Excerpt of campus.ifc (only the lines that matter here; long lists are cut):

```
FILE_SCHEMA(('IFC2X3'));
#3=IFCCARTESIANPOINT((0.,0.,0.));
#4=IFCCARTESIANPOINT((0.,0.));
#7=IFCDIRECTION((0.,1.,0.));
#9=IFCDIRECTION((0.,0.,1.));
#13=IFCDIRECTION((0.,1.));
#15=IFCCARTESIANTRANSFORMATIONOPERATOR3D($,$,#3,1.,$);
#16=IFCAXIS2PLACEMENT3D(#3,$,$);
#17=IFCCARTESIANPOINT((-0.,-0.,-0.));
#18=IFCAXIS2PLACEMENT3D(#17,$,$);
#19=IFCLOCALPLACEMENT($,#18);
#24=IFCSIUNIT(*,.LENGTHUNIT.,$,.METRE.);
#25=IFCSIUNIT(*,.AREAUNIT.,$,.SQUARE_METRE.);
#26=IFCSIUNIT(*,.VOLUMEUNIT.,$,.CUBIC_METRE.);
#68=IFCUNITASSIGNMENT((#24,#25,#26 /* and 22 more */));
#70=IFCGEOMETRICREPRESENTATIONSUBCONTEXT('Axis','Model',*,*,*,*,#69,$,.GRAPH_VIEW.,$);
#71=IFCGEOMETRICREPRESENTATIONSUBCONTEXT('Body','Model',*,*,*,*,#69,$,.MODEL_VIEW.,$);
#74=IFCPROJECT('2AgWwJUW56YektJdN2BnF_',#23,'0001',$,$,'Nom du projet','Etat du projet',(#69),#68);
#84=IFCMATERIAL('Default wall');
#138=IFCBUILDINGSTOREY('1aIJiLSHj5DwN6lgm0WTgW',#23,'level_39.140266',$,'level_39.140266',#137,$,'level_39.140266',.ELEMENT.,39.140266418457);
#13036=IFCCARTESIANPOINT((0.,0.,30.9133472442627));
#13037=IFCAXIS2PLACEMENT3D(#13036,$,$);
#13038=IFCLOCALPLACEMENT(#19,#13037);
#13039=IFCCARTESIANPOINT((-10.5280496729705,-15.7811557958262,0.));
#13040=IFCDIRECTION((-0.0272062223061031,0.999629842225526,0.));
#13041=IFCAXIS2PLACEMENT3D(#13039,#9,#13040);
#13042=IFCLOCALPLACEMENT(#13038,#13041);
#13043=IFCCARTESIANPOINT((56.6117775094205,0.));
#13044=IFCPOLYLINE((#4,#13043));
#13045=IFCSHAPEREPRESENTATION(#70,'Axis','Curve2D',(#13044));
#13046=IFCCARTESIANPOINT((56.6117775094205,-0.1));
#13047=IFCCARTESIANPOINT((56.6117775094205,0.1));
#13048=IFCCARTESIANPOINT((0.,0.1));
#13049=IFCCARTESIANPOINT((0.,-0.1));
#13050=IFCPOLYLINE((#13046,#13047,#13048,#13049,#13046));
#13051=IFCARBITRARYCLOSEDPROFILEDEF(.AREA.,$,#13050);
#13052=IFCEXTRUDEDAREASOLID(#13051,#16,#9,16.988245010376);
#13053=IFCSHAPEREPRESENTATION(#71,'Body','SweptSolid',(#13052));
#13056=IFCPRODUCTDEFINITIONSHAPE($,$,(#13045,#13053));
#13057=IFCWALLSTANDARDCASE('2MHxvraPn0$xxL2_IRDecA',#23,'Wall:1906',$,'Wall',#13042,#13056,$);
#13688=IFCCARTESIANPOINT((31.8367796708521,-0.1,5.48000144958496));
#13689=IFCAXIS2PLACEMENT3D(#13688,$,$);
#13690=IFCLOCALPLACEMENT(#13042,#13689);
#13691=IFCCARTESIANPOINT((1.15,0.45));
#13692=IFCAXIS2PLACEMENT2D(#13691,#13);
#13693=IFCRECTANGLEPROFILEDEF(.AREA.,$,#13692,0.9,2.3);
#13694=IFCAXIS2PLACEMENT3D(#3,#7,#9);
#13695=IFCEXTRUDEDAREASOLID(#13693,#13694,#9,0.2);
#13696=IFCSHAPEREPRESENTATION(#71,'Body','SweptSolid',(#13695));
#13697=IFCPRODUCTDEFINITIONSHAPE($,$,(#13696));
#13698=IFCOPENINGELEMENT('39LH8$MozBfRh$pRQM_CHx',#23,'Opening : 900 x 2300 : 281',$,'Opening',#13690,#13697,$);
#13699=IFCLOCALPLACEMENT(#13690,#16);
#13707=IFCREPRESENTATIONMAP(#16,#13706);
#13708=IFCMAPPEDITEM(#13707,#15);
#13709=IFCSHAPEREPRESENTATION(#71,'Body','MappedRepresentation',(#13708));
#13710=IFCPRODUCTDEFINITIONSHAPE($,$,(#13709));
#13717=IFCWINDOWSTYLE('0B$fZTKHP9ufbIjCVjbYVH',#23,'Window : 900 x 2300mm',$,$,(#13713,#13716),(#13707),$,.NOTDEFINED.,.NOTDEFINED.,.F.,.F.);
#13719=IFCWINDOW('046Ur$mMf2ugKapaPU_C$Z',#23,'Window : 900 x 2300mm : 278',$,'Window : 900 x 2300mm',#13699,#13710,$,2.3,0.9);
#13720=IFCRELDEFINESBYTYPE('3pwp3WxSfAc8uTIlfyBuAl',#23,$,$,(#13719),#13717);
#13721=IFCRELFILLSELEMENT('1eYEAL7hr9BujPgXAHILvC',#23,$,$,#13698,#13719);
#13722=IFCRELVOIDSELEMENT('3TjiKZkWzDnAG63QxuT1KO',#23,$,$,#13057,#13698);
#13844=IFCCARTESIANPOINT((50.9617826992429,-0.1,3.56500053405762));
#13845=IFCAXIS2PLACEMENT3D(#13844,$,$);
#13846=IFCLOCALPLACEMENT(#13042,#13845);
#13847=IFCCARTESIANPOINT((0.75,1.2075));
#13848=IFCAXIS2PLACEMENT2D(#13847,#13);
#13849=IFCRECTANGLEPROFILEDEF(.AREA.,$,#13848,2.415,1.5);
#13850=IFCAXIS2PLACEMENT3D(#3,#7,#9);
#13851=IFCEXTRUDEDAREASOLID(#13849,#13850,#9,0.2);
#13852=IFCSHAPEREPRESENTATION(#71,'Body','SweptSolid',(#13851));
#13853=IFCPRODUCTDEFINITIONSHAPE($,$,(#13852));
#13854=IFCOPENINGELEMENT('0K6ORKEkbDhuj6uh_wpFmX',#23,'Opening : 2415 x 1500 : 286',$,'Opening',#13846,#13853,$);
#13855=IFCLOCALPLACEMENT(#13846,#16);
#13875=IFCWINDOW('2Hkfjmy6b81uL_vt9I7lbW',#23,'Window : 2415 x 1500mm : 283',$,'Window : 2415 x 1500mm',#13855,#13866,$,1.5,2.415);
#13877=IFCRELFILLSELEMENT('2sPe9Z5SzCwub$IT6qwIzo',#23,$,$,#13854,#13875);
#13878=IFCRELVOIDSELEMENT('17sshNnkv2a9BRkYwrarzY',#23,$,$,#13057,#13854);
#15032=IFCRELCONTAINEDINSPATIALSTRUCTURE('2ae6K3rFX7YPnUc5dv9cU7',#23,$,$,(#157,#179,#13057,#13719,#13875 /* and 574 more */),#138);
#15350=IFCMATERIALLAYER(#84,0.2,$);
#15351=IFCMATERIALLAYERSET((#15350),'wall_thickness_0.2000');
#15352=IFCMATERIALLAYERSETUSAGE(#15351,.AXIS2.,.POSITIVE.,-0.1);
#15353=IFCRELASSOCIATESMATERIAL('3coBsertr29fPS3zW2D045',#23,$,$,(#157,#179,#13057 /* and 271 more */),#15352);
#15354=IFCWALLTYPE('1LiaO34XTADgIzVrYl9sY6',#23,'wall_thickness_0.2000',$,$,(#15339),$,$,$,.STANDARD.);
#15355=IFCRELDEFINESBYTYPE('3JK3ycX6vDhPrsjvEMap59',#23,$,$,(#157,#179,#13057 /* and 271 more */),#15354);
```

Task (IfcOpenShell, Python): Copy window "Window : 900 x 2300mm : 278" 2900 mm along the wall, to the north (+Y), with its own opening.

```python
import ifcopenshell
import ifcopenshell.api.feature
import ifcopenshell.api.geometry
import ifcopenshell.api.root
import ifcopenshell.geom
import ifcopenshell.util.element
import ifcopenshell.util.placement
import ifcopenshell.util.shape
import ifcopenshell.util.unit

model = ifcopenshell.open("campus.ifc")
unit_scale = ifcopenshell.util.unit.calculate_unit_scale(model)
settings = ifcopenshell.geom.settings()


def volume(element):
    """Net volume in cubic metres, openings subtracted."""
    shape = ifcopenshell.geom.create_shape(settings, element)
    return ifcopenshell.util.shape.get_volume(shape.geometry)


window = model.by_guid("046Ur$mMf2ugKapaPU_C$Z")
opening = window.FillsVoids[0].RelatingOpeningElement
wall = opening.VoidsElements[0].RelatingBuildingElement
before = volume(wall)
shift = ifcopenshell.util.placement.get_local_placement(wall.ObjectPlacement)[:3, 0] * 2.9 / unit_scale

# copy_class copies the void relationship, type, container and properties, but no geometry.
new_opening = ifcopenshell.api.root.copy_class(model, product=opening)
new_opening.Representation = ifcopenshell.util.element.copy_deep(
    model, opening.Representation, exclude=["IfcGeometricRepresentationContext", "IfcRepresentationMap"]
)
new_opening.Name = "Opening : 900 x 2300"
new_window = ifcopenshell.api.root.copy_class(model, product=window)
new_window.Representation = ifcopenshell.util.element.copy_deep(
    model, window.Representation, exclude=["IfcGeometricRepresentationContext", "IfcRepresentationMap"]
)
new_window.Name = "Window : 900 x 2300mm"
fills = ifcopenshell.api.feature.add_filling(model, opening=new_opening, element=new_window)
fills.OwnerHistory = new_window.OwnerHistory  # required in IFC2X3

for old, new in ((opening, new_opening), (window, new_window)):
    matrix = ifcopenshell.util.placement.get_local_placement(old.ObjectPlacement)
    matrix[:3, 3] += shift
    ifcopenshell.api.geometry.edit_object_placement(model, product=new, matrix=matrix, is_si=False)

after = volume(wall)

print(f"wall volume {before:.3f} -> {after:.3f} m3")

model.write("campus_edited.ifc")
```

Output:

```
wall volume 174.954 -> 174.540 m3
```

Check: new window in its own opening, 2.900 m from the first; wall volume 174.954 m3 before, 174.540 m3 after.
